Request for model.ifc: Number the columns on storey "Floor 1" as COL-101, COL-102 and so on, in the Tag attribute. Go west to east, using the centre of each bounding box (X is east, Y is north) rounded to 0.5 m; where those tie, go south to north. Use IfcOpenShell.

First a look at what the model holds.

```python
import ifcopenshell
import ifcopenshell.util.element
import ifcopenshell.util.placement

model = ifcopenshell.open("model.ifc")
print(model.schema)
storey = next(s for s in model.by_type("IfcBuildingStorey") if s.Name == "Floor 1")
columns = [e for e in ifcopenshell.util.element.get_decomposition(storey) if e.is_a("IfcColumn")]
for e in sorted(columns, key=lambda e: e.id()):
    origin = ifcopenshell.util.placement.get_local_placement(e.ObjectPlacement)[:3, 3]
    print(e.id(), e.Tag, e.Name, origin.round(2) + 0.0, sep=" | ")
```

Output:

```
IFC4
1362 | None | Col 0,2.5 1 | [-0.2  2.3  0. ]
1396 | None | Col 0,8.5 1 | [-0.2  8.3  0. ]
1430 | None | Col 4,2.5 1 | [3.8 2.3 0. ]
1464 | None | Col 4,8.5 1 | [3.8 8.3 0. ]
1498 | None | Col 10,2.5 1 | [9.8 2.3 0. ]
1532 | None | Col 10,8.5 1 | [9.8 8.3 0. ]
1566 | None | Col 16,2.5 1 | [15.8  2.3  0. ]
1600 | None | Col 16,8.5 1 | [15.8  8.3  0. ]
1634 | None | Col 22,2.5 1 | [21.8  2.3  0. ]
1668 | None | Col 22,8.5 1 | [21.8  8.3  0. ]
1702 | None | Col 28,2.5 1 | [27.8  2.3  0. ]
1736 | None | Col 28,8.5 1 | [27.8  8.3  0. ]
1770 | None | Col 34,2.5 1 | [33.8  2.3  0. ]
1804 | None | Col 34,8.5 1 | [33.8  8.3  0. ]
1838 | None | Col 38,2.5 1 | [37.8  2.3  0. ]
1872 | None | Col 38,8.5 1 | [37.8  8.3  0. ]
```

```python
import ifcopenshell
import ifcopenshell.geom
import ifcopenshell.util.element
import ifcopenshell.util.shape

model = ifcopenshell.open("model.ifc")
settings = ifcopenshell.geom.settings()
settings.set("use-world-coords", True)


def centre(element):
    shape = ifcopenshell.geom.create_shape(settings, element)
    return ifcopenshell.util.shape.get_bbox_centroid(shape.geometry)


storey = next(s for s in model.by_type("IfcBuildingStorey") if s.Name == "Floor 1")
columns = [e for e in ifcopenshell.util.element.get_decomposition(storey) if e.is_a("IfcColumn")]

# Insertion points can sit at a corner or the storey origin, so sort by the geometry (in metres).
centres = {e: centre(e) for e in columns}
columns.sort(key=lambda e: (round(centres[e][0] / 0.5), centres[e][1]))

for i, e in enumerate(columns, start=1):
    number = f"COL-1{i:02d}"
    e.Tag = number
    print(e.id(), number)

model.write("model_rev.ifc")
```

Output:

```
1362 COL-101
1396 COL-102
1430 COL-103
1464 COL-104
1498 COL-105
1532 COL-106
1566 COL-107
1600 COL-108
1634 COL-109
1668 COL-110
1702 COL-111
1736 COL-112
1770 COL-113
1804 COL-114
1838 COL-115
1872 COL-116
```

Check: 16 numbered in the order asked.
